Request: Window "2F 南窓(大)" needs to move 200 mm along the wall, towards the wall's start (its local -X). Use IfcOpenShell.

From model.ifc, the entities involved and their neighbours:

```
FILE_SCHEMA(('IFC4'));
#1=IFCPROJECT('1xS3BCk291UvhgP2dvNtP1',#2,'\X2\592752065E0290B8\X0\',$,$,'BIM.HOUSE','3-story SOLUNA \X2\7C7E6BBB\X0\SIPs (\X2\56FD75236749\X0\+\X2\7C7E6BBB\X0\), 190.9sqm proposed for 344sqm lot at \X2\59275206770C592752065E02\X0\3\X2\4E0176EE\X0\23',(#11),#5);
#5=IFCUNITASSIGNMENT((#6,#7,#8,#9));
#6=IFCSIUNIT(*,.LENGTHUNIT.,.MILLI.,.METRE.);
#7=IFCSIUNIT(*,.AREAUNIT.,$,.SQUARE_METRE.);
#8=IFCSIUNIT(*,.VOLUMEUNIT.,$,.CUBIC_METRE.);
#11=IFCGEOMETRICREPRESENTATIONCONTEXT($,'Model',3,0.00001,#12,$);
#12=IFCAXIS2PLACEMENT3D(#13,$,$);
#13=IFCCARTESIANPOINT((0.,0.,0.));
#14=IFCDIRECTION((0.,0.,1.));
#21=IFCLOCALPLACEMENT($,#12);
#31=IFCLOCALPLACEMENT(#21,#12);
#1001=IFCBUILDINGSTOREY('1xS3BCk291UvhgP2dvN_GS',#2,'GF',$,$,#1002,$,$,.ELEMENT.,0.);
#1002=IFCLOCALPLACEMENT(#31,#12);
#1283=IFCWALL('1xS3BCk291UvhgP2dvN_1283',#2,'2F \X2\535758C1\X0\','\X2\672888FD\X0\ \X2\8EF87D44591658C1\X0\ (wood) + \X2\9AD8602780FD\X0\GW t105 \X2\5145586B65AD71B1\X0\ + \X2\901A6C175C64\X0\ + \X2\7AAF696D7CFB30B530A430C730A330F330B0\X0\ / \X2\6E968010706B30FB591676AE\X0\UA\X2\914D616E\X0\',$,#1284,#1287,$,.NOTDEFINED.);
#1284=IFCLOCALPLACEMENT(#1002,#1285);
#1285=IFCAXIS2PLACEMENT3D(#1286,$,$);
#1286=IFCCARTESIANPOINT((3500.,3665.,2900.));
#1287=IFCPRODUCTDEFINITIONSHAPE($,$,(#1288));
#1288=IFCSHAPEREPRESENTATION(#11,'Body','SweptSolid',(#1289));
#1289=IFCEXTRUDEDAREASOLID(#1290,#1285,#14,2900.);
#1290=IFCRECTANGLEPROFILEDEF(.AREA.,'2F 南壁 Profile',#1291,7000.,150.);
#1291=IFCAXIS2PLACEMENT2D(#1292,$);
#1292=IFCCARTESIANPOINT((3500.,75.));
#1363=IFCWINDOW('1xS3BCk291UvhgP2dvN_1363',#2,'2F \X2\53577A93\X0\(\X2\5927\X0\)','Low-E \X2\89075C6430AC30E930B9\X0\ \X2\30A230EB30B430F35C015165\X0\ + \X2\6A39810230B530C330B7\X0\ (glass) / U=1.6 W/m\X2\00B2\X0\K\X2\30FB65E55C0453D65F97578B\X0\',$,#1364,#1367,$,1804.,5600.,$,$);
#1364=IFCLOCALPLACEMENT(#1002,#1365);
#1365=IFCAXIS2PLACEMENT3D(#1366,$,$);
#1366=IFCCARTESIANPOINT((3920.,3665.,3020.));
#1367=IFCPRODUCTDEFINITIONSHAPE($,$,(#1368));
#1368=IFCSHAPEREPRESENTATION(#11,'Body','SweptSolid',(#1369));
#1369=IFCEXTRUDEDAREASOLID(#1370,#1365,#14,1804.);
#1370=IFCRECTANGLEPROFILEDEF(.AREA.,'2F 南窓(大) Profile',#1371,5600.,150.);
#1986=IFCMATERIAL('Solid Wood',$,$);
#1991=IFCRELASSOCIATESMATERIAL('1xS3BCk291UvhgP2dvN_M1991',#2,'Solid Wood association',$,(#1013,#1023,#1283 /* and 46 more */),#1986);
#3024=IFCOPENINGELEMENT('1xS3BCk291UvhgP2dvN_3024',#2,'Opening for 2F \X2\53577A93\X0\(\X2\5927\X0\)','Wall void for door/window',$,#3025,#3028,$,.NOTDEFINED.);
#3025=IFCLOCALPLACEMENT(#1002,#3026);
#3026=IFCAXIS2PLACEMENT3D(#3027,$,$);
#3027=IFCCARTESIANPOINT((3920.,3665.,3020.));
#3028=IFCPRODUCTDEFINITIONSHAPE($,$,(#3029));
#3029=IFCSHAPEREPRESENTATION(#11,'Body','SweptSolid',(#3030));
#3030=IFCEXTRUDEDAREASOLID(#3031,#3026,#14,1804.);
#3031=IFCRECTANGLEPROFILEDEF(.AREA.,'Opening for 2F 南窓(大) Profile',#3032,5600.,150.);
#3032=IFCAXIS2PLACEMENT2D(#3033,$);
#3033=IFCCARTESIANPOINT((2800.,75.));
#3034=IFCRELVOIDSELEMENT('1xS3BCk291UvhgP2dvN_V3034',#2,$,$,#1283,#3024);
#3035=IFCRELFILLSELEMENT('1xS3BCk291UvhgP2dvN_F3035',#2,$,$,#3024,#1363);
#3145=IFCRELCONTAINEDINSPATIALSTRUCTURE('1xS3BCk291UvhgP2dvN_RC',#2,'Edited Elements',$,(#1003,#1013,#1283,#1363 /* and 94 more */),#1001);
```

```python
import ifcopenshell
import ifcopenshell.api.geometry
import ifcopenshell.util.placement

model = ifcopenshell.open("model.ifc")

window = model.by_guid("1xS3BCk291UvhgP2dvN_1363")
opening = window.FillsVoids[0].RelatingOpeningElement
wall = opening.VoidsElements[0].RelatingBuildingElement

wall_matrix = ifcopenshell.util.placement.get_local_placement(wall.ObjectPlacement)
shift = wall_matrix[:3, 0] * -200.0
before = ifcopenshell.util.placement.get_local_placement(window.ObjectPlacement)[:3, 3].copy()

# The window is not placed relative to its opening, so move both.
for product in (opening, window):
    matrix = ifcopenshell.util.placement.get_local_placement(product.ObjectPlacement)
    matrix[:3, 3] += shift
    ifcopenshell.api.geometry.edit_object_placement(model, product=product, matrix=matrix, is_si=False)

after = ifcopenshell.util.placement.get_local_placement(window.ObjectPlacement)[:3, 3]
print("window moved by", (after - before).round(3) + 0.0)

model.write("model-out.ifc")
```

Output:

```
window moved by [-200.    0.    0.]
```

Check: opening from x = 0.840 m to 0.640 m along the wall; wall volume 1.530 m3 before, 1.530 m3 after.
